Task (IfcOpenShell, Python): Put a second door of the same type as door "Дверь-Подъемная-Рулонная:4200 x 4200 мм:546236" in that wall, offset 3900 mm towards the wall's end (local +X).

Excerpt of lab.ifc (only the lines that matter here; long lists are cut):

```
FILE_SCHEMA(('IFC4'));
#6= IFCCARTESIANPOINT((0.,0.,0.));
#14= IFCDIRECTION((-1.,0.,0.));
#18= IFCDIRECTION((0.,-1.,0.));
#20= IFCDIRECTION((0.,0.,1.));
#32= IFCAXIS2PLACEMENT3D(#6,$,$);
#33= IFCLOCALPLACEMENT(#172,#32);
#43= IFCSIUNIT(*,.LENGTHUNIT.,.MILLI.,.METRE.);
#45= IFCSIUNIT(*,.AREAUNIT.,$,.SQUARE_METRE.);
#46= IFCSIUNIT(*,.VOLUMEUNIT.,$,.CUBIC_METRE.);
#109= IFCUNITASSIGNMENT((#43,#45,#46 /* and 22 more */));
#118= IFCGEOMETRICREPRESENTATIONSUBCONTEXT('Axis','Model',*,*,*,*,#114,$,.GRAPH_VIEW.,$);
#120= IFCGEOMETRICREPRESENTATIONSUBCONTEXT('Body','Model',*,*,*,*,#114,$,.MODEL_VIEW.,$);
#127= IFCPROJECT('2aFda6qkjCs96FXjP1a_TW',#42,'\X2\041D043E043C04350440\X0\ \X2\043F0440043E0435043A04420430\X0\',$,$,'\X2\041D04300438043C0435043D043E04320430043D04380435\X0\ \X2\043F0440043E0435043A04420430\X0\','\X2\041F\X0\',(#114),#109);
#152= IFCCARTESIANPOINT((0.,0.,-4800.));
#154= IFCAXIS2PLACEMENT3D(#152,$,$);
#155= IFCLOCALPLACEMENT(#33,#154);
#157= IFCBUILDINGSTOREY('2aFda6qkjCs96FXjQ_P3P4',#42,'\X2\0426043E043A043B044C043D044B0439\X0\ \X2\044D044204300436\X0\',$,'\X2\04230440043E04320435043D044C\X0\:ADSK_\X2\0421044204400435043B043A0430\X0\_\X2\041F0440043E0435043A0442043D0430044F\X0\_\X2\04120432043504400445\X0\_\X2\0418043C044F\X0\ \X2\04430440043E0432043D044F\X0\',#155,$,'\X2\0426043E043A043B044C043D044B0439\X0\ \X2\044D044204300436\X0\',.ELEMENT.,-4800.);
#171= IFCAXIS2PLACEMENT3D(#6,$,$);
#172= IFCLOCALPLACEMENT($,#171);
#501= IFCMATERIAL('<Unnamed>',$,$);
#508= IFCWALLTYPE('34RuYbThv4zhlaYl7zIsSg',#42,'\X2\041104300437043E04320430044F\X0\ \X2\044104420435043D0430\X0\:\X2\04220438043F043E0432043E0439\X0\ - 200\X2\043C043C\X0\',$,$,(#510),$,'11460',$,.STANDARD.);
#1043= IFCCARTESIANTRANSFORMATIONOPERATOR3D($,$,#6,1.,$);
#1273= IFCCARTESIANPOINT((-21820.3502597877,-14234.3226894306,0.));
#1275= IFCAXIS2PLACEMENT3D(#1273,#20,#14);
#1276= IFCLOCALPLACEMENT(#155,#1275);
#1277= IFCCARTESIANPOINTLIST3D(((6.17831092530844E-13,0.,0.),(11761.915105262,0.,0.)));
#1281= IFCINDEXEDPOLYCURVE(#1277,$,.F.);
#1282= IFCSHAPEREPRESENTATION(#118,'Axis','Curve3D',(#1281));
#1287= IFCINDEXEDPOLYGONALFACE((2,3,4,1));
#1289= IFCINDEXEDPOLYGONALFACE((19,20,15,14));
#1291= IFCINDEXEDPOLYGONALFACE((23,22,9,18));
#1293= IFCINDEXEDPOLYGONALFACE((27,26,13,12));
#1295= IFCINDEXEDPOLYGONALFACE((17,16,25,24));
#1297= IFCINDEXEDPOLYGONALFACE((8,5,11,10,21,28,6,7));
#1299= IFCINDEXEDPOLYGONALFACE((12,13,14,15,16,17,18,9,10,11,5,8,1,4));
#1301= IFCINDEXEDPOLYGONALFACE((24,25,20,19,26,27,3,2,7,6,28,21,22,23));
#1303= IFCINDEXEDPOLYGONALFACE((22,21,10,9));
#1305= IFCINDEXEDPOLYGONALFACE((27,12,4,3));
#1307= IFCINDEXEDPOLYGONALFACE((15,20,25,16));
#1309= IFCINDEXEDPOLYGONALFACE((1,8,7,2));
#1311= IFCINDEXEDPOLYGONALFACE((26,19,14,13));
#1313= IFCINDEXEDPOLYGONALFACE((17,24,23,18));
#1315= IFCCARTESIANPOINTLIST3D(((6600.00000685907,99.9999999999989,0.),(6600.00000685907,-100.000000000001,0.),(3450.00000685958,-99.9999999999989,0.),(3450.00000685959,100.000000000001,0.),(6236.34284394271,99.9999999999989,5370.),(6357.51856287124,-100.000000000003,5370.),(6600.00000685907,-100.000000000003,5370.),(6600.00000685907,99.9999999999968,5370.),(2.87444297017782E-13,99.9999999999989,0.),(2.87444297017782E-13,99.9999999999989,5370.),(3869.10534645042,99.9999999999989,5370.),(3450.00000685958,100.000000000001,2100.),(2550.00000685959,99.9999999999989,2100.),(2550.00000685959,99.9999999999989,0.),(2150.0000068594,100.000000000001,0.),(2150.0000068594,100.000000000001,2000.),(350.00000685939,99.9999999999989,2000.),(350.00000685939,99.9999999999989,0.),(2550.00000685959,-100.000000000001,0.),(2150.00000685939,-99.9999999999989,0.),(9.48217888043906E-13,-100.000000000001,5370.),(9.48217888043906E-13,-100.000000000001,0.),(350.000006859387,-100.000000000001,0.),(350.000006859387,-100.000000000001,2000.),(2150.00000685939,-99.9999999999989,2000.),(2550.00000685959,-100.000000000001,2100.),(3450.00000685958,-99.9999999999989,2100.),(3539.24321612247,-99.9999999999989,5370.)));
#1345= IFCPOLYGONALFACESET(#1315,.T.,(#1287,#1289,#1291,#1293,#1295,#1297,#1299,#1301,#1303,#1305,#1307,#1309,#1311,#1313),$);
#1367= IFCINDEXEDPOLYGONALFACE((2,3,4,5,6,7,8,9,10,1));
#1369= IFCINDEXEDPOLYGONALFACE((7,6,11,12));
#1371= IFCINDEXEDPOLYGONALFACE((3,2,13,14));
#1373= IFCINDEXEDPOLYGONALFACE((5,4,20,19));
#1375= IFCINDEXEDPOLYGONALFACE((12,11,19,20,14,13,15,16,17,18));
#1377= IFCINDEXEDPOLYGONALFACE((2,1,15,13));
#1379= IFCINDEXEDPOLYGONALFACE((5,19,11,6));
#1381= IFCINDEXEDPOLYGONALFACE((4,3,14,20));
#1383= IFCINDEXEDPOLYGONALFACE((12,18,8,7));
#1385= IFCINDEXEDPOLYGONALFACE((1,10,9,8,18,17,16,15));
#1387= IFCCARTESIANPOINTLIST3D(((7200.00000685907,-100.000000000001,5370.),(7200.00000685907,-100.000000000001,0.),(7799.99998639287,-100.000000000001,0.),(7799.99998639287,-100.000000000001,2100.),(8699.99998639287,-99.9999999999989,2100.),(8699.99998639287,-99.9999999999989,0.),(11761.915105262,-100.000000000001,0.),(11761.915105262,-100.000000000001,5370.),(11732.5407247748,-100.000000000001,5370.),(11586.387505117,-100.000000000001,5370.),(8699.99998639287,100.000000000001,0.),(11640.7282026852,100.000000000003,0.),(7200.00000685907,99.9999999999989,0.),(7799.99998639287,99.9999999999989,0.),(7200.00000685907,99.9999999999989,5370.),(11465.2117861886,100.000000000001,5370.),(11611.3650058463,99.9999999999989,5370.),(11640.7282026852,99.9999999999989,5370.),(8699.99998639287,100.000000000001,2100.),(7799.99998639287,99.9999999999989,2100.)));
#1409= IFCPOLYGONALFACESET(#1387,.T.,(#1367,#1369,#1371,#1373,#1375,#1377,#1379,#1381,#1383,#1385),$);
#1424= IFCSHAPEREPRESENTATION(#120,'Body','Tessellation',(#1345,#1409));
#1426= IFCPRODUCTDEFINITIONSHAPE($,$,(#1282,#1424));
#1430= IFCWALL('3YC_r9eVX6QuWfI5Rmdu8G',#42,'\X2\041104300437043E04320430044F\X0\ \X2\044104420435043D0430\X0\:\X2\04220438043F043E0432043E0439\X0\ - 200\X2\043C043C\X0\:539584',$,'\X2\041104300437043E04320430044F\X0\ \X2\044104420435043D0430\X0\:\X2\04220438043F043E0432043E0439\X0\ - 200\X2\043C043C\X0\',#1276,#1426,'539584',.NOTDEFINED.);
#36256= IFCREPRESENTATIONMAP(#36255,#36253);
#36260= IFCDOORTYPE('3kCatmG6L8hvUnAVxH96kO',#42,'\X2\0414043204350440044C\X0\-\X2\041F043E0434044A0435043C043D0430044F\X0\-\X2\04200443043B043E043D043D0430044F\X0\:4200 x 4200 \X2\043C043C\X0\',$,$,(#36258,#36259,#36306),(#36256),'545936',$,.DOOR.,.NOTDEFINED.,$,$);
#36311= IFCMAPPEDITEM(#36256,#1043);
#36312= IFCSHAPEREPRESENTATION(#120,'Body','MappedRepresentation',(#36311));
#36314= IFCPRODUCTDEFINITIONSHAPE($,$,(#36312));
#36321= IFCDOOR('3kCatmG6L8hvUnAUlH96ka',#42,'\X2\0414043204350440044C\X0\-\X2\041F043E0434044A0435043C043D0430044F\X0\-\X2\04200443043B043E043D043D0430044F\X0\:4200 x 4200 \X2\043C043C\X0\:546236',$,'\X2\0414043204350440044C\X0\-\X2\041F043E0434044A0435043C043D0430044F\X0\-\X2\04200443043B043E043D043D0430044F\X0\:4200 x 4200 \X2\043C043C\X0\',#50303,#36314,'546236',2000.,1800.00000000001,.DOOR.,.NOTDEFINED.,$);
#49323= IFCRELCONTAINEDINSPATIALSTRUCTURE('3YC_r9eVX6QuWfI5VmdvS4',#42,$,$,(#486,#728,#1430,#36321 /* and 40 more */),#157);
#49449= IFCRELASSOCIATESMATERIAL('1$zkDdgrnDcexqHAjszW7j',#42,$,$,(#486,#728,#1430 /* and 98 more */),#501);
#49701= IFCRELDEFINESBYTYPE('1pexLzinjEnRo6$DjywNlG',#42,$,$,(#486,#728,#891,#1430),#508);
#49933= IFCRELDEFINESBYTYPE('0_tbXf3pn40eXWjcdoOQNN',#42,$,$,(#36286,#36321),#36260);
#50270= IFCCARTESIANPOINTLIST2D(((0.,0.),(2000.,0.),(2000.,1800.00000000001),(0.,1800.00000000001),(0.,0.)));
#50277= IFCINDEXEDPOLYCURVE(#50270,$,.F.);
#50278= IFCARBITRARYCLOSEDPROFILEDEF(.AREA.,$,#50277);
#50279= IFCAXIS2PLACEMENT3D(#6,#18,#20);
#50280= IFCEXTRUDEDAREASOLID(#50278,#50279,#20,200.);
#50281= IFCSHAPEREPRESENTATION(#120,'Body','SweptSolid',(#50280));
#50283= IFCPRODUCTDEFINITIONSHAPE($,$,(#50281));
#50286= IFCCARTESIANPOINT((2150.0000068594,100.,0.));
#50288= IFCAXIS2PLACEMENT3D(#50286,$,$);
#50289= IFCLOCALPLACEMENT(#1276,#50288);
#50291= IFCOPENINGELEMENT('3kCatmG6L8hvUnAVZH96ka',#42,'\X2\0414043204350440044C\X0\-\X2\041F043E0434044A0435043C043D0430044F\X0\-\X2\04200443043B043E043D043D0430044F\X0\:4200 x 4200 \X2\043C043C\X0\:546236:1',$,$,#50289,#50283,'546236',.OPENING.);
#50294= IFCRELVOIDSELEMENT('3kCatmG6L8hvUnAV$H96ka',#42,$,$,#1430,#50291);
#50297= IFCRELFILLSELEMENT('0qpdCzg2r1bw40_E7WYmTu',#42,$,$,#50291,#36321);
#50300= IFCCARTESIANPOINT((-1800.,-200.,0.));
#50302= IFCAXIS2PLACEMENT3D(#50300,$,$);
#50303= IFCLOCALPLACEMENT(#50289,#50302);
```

```python
import ifcopenshell
import ifcopenshell.api.feature
import ifcopenshell.api.geometry
import ifcopenshell.api.root
import ifcopenshell.geom
import ifcopenshell.util.element
import ifcopenshell.util.placement
import ifcopenshell.util.shape

model = ifcopenshell.open("lab.ifc")
settings = ifcopenshell.geom.settings()


def volume(element):
    """Net volume in cubic metres, openings subtracted."""
    shape = ifcopenshell.geom.create_shape(settings, element)
    return ifcopenshell.util.shape.get_volume(shape.geometry)


def reuse_history(source, copy):
    """copy_class also copies each property set's owner history, people and application; keep the originals."""
    for rel in copy.IsDefinedBy:
        if rel.is_a("IfcRelDefinesByProperties") and (history := rel.RelatingPropertyDefinition.OwnerHistory):
            rel.RelatingPropertyDefinition.OwnerHistory = source.OwnerHistory
            ifcopenshell.util.element.remove_deep2(model, history)


door = model.by_guid("3kCatmG6L8hvUnAUlH96ka")
opening = door.FillsVoids[0].RelatingOpeningElement
wall = opening.VoidsElements[0].RelatingBuildingElement
before = volume(wall)
shift = ifcopenshell.util.placement.get_local_placement(wall.ObjectPlacement)[:3, 0] * 3900.0

# copy_class copies the void relationship, type, container and properties, but no geometry.
new_opening = ifcopenshell.api.root.copy_class(model, product=opening)
new_opening.Representation = ifcopenshell.util.element.copy_deep(
    model, opening.Representation, exclude=["IfcGeometricRepresentationContext", "IfcRepresentationMap"]
)
new_opening.Name = "Дверь-Подъемная-Рулонная:4200 x 4200 мм"
new_opening.Tag = None
new_door = ifcopenshell.api.root.copy_class(model, product=door)
new_door.Representation = ifcopenshell.util.element.copy_deep(
    model, door.Representation, exclude=["IfcGeometricRepresentationContext", "IfcRepresentationMap"]
)
new_door.Name = "Дверь-Подъемная-Рулонная:4200 x 4200 мм"
new_door.Tag = None
reuse_history(door, new_door)
ifcopenshell.api.feature.add_filling(model, opening=new_opening, element=new_door)

for old, new in ((opening, new_opening), (door, new_door)):
    matrix = ifcopenshell.util.placement.get_local_placement(old.ObjectPlacement)
    matrix[:3, 3] += shift
    ifcopenshell.api.geometry.edit_object_placement(model, product=new, matrix=matrix, is_si=False)

after = volume(wall)

print(f"wall volume {before:.3f} -> {after:.3f} m3")

model.write("lab_edited.ifc")
```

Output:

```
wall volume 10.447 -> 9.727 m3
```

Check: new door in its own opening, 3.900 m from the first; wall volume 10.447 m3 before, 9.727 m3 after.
